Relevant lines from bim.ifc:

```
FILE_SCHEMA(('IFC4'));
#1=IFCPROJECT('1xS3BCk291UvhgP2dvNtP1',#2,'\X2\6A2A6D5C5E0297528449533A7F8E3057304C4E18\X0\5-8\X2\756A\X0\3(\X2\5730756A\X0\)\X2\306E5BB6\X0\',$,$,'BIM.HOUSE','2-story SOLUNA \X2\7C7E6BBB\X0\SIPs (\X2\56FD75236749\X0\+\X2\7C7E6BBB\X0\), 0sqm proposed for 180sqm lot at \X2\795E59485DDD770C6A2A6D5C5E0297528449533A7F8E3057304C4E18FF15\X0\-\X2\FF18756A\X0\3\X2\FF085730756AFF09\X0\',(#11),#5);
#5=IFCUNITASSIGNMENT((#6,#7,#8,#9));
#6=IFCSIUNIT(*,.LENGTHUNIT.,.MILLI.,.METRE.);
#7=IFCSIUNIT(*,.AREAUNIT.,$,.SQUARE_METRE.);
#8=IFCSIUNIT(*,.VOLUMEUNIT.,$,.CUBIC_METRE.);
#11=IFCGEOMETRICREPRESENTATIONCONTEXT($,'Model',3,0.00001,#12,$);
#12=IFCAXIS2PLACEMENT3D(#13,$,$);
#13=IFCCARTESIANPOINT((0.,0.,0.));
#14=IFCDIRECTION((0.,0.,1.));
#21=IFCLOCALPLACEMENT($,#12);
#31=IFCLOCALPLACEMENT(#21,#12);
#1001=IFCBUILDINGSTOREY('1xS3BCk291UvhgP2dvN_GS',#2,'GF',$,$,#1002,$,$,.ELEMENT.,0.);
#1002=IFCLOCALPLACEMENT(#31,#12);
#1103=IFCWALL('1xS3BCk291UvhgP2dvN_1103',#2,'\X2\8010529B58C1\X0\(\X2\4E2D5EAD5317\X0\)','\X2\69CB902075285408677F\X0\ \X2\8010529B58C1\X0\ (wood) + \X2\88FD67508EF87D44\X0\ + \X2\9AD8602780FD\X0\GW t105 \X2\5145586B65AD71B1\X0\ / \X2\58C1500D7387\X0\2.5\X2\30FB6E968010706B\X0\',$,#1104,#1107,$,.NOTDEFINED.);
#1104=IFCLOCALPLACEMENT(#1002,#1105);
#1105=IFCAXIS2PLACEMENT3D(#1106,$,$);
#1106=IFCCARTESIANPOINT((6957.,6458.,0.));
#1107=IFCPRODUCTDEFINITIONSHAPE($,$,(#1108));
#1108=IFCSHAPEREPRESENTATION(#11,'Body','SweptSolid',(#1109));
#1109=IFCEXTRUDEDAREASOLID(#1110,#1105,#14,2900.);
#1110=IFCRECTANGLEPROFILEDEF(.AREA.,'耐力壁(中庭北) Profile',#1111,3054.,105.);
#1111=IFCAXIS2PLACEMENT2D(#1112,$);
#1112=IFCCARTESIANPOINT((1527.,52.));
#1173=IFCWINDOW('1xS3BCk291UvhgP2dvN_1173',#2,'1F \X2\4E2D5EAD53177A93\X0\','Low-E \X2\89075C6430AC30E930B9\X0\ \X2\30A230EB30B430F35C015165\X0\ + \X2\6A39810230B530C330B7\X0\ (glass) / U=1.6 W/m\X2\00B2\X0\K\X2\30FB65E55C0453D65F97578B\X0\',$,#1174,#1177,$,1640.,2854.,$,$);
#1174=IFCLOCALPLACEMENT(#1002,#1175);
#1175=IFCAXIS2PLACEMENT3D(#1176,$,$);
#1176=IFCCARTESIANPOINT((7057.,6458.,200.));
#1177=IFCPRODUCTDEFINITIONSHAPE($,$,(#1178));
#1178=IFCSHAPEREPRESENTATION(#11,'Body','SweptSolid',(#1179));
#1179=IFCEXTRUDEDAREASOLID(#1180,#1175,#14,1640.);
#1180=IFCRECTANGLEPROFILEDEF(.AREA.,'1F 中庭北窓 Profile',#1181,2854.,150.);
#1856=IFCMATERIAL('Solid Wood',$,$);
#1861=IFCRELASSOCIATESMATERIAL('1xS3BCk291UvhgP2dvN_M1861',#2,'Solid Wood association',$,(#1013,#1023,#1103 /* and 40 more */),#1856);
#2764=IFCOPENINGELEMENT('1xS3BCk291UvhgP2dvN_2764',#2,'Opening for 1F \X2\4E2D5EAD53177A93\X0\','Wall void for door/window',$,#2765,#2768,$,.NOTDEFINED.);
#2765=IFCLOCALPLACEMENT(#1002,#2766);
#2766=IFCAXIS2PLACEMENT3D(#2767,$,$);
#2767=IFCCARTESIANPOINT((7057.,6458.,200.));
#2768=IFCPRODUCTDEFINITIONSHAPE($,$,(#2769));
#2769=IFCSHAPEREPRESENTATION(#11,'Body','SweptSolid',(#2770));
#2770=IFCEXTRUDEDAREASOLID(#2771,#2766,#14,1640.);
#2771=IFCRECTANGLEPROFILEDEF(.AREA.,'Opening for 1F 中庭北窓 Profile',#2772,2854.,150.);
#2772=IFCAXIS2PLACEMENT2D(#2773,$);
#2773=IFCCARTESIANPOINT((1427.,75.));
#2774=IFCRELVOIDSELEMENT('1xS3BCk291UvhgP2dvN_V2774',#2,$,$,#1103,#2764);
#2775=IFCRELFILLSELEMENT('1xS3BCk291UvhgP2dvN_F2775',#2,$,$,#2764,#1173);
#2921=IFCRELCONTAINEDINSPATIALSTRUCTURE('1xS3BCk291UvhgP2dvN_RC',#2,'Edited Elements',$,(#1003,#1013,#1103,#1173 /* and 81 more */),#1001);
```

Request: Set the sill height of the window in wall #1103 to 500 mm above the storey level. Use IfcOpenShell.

```python
import numpy as np
import ifcopenshell
import ifcopenshell.api.geometry
import ifcopenshell.geom
import ifcopenshell.util.element
import ifcopenshell.util.placement
import ifcopenshell.util.shape
import ifcopenshell.util.unit

model = ifcopenshell.open("bim.ifc")
unit_scale = ifcopenshell.util.unit.calculate_unit_scale(model)

window = model.by_guid("1xS3BCk291UvhgP2dvN_1173")
opening = window.FillsVoids[0].RelatingOpeningElement
storey = ifcopenshell.util.element.get_container(window, ifc_class="IfcBuildingStorey")
level = ifcopenshell.util.placement.get_local_placement(storey.ObjectPlacement)[2, 3]

# The opening's origin need not be at the sill, so measure its lowest point.
shape = ifcopenshell.geom.create_shape(ifcopenshell.geom.settings(), opening)
bottom = ifcopenshell.util.shape.get_shape_bottom_elevation(shape, shape.geometry) / unit_scale
dz = level + 0.5 / unit_scale - bottom

shift = np.array([0.0, 0.0, dz])
# The window is not placed relative to its opening, so move both.
for product in (opening, window):
    matrix = ifcopenshell.util.placement.get_local_placement(product.ObjectPlacement)
    matrix[:3, 3] += shift
    ifcopenshell.api.geometry.edit_object_placement(model, product=product, matrix=matrix, is_si=False)

print(f"moved by {dz * unit_scale:+.3f} m")

model.write("bim-out.ifc")
```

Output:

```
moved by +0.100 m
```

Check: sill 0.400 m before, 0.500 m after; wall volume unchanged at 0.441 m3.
